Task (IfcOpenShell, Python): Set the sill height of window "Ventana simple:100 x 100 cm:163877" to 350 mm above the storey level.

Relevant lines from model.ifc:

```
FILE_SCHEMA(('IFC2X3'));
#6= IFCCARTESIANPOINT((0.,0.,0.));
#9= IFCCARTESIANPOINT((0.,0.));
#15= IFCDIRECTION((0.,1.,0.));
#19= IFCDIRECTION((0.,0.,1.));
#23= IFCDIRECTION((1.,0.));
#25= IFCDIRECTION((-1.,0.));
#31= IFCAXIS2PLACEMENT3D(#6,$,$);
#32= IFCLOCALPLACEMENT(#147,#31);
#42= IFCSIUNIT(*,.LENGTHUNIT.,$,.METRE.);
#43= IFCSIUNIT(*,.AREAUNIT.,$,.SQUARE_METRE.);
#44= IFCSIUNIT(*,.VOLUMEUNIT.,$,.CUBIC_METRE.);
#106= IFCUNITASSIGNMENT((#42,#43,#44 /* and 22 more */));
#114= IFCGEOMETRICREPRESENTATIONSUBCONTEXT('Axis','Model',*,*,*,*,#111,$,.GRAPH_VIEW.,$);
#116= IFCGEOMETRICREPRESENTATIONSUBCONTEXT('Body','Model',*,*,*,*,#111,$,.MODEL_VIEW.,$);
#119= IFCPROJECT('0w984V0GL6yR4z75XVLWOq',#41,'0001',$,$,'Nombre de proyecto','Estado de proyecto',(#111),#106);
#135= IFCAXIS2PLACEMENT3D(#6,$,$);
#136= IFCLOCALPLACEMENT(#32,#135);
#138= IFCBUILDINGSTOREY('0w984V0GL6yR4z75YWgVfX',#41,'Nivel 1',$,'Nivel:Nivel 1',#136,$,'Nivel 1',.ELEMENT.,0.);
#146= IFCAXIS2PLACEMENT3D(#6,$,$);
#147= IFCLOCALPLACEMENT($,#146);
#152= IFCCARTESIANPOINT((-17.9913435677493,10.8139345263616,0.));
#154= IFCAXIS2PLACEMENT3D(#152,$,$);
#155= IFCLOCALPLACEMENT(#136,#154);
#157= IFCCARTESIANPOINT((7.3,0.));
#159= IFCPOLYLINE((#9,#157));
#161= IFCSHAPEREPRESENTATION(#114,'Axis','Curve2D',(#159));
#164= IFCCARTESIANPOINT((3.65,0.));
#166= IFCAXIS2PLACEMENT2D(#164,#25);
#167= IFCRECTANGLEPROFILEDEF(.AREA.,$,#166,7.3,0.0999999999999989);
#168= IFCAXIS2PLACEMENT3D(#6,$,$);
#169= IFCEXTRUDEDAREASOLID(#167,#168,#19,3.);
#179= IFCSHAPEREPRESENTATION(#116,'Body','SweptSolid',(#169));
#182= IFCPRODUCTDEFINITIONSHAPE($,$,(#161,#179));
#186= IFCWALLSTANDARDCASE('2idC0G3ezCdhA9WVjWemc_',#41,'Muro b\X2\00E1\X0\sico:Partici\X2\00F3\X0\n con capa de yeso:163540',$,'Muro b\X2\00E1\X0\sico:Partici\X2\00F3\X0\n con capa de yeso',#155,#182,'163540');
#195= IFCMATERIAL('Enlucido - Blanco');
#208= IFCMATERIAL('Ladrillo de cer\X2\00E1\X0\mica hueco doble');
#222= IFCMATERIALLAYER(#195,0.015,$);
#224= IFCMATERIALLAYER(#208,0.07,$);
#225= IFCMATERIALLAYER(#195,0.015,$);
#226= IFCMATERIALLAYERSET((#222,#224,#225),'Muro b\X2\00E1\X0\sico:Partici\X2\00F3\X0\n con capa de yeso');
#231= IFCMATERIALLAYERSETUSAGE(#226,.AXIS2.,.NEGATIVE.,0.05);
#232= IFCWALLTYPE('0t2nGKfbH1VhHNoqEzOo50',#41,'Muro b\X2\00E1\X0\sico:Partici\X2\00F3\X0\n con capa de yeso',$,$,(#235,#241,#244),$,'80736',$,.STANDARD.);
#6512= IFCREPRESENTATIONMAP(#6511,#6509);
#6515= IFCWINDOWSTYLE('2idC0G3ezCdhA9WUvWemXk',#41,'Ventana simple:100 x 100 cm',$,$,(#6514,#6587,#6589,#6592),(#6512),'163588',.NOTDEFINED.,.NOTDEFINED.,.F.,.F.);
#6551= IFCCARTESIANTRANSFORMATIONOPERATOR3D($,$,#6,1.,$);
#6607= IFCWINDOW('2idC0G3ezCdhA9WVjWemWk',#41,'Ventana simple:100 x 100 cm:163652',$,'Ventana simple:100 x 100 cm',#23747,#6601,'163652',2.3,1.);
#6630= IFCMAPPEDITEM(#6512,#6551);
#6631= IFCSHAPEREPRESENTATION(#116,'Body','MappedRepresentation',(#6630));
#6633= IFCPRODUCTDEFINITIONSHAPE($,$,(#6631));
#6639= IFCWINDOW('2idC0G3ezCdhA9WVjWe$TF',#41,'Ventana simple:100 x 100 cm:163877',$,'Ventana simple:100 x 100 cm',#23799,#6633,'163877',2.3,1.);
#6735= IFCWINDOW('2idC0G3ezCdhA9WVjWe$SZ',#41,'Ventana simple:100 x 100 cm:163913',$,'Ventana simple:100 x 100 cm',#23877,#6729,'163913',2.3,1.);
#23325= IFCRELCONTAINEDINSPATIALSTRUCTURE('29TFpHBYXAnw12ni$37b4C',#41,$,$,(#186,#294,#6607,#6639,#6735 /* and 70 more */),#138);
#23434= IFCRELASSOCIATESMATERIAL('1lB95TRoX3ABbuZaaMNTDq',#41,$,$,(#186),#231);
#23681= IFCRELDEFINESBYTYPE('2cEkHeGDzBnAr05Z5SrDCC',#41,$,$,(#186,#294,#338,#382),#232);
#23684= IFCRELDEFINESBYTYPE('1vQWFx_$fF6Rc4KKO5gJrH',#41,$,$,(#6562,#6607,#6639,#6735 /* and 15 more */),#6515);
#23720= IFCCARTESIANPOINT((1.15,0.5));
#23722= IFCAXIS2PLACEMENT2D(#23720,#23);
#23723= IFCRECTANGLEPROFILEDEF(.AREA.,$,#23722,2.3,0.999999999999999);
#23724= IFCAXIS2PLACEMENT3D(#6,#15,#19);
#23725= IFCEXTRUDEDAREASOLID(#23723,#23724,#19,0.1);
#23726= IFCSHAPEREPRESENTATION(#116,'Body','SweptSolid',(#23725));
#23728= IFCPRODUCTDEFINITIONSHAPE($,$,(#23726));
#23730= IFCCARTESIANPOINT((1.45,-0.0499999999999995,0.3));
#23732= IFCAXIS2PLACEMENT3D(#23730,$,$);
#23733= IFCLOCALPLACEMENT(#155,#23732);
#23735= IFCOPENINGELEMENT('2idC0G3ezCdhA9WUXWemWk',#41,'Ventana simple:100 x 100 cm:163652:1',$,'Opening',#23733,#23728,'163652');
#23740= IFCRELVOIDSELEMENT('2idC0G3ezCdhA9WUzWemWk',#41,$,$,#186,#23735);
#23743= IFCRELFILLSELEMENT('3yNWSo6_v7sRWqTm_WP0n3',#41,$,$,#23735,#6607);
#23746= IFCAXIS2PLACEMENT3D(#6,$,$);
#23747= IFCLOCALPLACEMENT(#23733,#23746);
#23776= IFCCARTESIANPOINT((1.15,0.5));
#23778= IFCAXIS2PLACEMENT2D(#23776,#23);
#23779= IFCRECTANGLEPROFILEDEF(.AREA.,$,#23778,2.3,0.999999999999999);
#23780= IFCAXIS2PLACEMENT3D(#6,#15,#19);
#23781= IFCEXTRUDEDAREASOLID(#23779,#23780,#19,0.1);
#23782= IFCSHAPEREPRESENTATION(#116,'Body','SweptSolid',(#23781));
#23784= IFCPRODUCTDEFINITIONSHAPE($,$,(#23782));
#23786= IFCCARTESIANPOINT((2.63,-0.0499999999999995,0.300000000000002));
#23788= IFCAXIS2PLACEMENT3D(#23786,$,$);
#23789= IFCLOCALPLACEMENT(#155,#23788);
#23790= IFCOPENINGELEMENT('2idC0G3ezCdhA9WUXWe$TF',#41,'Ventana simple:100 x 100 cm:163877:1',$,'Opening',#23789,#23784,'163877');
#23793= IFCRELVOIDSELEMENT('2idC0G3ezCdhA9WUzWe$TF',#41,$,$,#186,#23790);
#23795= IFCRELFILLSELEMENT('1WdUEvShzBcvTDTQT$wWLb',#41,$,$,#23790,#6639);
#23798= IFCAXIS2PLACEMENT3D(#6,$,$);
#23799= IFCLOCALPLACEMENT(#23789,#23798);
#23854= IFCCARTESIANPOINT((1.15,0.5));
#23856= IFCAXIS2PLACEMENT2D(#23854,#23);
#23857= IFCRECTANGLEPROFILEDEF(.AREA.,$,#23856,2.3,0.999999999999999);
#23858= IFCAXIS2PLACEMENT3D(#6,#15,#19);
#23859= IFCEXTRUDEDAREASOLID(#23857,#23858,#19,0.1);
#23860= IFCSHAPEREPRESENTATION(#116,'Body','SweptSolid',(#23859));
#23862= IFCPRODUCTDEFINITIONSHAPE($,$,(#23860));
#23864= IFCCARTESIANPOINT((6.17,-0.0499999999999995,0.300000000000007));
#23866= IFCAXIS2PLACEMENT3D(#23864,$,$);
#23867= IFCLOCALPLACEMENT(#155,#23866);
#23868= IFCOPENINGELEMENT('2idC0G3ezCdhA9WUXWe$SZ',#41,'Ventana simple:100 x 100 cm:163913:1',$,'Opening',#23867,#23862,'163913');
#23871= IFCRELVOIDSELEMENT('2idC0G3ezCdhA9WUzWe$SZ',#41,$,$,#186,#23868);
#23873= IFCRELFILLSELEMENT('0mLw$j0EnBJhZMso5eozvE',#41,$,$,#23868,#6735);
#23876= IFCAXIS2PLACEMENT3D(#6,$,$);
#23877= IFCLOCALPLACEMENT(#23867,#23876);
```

```python
import numpy as np
import ifcopenshell
import ifcopenshell.api.geometry
import ifcopenshell.geom
import ifcopenshell.util.element
import ifcopenshell.util.placement
import ifcopenshell.util.shape
import ifcopenshell.util.unit

model = ifcopenshell.open("model.ifc")
unit_scale = ifcopenshell.util.unit.calculate_unit_scale(model)

window = model.by_id(6639)
opening = window.FillsVoids[0].RelatingOpeningElement
storey = ifcopenshell.util.element.get_container(window, ifc_class="IfcBuildingStorey")
level = ifcopenshell.util.placement.get_local_placement(storey.ObjectPlacement)[2, 3]

# The opening's origin need not be at the sill, so measure its lowest point.
shape = ifcopenshell.geom.create_shape(ifcopenshell.geom.settings(), opening)
bottom = ifcopenshell.util.shape.get_shape_bottom_elevation(shape, shape.geometry) / unit_scale
dz = level + 0.35 / unit_scale - bottom

shift = np.array([0.0, 0.0, dz])
# The window is placed relative to its opening, so it follows when the opening moves.
matrix = ifcopenshell.util.placement.get_local_placement(opening.ObjectPlacement)
matrix[:3, 3] += shift
ifcopenshell.api.geometry.edit_object_placement(
    model, product=opening, matrix=matrix, is_si=False, should_transform_children=True
)

print(f"moved by {dz * unit_scale:+.3f} m")

model.write("model_v2.ifc")
```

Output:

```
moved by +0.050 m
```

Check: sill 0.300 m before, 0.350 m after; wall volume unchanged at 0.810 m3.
